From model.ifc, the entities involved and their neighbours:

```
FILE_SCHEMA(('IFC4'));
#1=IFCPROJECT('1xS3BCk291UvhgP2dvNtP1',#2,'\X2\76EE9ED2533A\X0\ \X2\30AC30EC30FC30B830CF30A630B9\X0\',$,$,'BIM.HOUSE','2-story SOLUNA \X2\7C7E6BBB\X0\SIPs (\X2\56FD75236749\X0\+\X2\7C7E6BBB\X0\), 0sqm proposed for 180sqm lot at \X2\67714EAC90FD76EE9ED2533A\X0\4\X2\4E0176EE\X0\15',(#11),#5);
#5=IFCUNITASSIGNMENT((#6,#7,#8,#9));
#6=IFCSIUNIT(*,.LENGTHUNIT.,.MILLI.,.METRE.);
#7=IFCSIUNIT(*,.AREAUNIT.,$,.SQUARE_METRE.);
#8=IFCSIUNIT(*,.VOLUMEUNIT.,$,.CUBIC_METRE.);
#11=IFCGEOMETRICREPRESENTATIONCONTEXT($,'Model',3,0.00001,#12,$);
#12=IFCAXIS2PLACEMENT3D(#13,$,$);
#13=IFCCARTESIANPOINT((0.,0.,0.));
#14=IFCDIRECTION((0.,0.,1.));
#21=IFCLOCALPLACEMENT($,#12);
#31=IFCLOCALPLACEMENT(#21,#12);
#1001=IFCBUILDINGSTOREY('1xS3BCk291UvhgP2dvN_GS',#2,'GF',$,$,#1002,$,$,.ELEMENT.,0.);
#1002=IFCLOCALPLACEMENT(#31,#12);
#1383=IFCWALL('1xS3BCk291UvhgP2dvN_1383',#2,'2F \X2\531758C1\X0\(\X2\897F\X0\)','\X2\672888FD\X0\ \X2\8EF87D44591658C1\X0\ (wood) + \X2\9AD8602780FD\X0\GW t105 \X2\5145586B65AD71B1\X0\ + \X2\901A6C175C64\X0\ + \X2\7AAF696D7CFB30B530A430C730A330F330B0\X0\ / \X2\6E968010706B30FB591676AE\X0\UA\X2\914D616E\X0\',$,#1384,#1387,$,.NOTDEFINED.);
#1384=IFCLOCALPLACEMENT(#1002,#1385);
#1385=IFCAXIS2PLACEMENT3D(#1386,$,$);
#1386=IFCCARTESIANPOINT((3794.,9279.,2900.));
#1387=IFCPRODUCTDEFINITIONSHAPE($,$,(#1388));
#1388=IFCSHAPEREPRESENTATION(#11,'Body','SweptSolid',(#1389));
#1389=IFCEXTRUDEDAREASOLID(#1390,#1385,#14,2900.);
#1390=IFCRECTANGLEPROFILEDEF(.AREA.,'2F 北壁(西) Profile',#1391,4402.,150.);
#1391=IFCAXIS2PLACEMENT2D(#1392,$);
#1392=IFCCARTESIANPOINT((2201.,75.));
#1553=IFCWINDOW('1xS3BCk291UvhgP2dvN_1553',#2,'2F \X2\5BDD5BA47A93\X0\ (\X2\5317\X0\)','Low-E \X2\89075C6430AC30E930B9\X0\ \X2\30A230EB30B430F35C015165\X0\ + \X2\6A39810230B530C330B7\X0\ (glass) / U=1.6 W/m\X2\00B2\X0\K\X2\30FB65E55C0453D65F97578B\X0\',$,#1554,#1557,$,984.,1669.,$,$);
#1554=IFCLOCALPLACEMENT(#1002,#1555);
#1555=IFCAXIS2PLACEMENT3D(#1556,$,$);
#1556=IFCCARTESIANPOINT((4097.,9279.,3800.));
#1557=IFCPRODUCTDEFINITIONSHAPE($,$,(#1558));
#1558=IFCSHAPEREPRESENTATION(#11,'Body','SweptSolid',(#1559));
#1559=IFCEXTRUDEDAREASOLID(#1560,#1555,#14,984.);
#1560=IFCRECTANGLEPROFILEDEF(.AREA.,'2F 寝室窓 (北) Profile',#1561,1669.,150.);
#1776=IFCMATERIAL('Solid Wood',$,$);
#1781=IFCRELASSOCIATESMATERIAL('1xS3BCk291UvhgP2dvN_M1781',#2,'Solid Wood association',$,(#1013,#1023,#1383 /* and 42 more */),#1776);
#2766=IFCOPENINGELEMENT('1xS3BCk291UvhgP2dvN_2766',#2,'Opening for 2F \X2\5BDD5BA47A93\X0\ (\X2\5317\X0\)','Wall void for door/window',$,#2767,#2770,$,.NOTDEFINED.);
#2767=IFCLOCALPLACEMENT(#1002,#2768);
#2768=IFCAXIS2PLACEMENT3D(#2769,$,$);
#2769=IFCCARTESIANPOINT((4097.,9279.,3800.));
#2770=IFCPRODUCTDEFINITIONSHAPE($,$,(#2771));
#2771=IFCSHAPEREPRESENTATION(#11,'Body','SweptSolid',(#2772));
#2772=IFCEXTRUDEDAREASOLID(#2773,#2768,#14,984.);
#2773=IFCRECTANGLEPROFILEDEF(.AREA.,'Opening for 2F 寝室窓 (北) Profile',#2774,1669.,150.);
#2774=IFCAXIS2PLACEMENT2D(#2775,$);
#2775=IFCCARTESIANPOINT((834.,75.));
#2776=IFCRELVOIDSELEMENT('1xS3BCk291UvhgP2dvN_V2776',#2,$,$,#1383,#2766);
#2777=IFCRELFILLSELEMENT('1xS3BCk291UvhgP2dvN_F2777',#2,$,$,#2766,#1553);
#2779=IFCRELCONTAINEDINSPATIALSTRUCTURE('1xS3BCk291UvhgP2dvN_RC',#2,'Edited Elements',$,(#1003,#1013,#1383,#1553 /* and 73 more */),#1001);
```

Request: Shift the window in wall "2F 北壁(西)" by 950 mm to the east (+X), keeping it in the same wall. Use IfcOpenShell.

```python
import ifcopenshell
import ifcopenshell.api.geometry
import ifcopenshell.util.placement

model = ifcopenshell.open("model.ifc")

window = model.by_guid("1xS3BCk291UvhgP2dvN_1553")
opening = window.FillsVoids[0].RelatingOpeningElement
wall = opening.VoidsElements[0].RelatingBuildingElement

wall_matrix = ifcopenshell.util.placement.get_local_placement(wall.ObjectPlacement)
shift = wall_matrix[:3, 0] * 950.0
before = ifcopenshell.util.placement.get_local_placement(window.ObjectPlacement)[:3, 3].copy()

# The window is not placed relative to its opening, so move both.
for product in (opening, window):
    matrix = ifcopenshell.util.placement.get_local_placement(product.ObjectPlacement)
    matrix[:3, 3] += shift
    ifcopenshell.api.geometry.edit_object_placement(model, product=product, matrix=matrix, is_si=False)

after = ifcopenshell.util.placement.get_local_placement(window.ObjectPlacement)[:3, 3]
print("window moved by", (after - before).round(3) + 0.0)

model.write("model_edited.ifc")
```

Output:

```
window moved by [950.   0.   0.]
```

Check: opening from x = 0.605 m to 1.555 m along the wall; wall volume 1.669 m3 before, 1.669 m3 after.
